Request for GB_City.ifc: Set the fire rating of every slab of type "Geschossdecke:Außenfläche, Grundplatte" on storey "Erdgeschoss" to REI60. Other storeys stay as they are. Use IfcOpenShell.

First a look at what the model holds.

```python
import ifcopenshell
import ifcopenshell.util.element

model = ifcopenshell.open("GB_City.ifc")
print(model.schema)
storey = next(s for s in model.by_type("IfcBuildingStorey") if s.Name == "Erdgeschoss")
slabs = [e for e in ifcopenshell.util.element.get_decomposition(storey) if e.is_a("IfcSlab")]
seen = {}
for e in slabs:
    element_type = ifcopenshell.util.element.get_type(e)
    key = (element_type.Name if element_type != e and element_type else None, ifcopenshell.util.element.get_pset(e, "Pset_SlabCommon", "FireRating"))
    seen[key] = seen.get(key, 0) + 1
for (name, value), count in sorted(seen.items(), key=str):
    print(count, "x", name, "|", value)
```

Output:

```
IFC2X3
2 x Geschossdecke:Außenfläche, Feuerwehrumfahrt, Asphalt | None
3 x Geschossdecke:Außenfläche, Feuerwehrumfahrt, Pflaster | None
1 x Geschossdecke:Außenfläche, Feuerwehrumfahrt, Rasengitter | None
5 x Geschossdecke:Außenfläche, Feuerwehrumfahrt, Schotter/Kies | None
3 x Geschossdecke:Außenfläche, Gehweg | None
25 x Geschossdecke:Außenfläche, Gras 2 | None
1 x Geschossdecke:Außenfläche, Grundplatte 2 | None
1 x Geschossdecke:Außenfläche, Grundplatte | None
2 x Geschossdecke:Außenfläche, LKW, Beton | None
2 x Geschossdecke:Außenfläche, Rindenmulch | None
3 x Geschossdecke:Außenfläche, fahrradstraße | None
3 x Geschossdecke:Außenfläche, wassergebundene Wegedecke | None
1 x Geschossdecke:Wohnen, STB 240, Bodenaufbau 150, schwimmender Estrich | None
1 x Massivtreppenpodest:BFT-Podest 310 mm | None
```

```python
import ifcopenshell
import ifcopenshell.api.pset
import ifcopenshell.util.element

model = ifcopenshell.open("GB_City.ifc")

storey = next(s for s in model.by_type("IfcBuildingStorey") if s.Name == "Erdgeschoss")
slabs = [e for e in ifcopenshell.util.element.get_decomposition(storey) if e.is_a("IfcSlab")]

count = 0
for e in slabs:
    element_type = ifcopenshell.util.element.get_type(e)
    if element_type in (None, e) or element_type.Name != "Geschossdecke:Außenfläche, Grundplatte":
        continue
    # add_pset returns the element's existing set when there is one.
    pset = ifcopenshell.api.pset.add_pset(model, product=e, name="Pset_SlabCommon")
    ifcopenshell.api.pset.edit_pset(model, pset=pset, properties={"FireRating": "REI60"})
    count += 1

print(count, "slabs updated")

model.write("GB_City_edited.ifc")
```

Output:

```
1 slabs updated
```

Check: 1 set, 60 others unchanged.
